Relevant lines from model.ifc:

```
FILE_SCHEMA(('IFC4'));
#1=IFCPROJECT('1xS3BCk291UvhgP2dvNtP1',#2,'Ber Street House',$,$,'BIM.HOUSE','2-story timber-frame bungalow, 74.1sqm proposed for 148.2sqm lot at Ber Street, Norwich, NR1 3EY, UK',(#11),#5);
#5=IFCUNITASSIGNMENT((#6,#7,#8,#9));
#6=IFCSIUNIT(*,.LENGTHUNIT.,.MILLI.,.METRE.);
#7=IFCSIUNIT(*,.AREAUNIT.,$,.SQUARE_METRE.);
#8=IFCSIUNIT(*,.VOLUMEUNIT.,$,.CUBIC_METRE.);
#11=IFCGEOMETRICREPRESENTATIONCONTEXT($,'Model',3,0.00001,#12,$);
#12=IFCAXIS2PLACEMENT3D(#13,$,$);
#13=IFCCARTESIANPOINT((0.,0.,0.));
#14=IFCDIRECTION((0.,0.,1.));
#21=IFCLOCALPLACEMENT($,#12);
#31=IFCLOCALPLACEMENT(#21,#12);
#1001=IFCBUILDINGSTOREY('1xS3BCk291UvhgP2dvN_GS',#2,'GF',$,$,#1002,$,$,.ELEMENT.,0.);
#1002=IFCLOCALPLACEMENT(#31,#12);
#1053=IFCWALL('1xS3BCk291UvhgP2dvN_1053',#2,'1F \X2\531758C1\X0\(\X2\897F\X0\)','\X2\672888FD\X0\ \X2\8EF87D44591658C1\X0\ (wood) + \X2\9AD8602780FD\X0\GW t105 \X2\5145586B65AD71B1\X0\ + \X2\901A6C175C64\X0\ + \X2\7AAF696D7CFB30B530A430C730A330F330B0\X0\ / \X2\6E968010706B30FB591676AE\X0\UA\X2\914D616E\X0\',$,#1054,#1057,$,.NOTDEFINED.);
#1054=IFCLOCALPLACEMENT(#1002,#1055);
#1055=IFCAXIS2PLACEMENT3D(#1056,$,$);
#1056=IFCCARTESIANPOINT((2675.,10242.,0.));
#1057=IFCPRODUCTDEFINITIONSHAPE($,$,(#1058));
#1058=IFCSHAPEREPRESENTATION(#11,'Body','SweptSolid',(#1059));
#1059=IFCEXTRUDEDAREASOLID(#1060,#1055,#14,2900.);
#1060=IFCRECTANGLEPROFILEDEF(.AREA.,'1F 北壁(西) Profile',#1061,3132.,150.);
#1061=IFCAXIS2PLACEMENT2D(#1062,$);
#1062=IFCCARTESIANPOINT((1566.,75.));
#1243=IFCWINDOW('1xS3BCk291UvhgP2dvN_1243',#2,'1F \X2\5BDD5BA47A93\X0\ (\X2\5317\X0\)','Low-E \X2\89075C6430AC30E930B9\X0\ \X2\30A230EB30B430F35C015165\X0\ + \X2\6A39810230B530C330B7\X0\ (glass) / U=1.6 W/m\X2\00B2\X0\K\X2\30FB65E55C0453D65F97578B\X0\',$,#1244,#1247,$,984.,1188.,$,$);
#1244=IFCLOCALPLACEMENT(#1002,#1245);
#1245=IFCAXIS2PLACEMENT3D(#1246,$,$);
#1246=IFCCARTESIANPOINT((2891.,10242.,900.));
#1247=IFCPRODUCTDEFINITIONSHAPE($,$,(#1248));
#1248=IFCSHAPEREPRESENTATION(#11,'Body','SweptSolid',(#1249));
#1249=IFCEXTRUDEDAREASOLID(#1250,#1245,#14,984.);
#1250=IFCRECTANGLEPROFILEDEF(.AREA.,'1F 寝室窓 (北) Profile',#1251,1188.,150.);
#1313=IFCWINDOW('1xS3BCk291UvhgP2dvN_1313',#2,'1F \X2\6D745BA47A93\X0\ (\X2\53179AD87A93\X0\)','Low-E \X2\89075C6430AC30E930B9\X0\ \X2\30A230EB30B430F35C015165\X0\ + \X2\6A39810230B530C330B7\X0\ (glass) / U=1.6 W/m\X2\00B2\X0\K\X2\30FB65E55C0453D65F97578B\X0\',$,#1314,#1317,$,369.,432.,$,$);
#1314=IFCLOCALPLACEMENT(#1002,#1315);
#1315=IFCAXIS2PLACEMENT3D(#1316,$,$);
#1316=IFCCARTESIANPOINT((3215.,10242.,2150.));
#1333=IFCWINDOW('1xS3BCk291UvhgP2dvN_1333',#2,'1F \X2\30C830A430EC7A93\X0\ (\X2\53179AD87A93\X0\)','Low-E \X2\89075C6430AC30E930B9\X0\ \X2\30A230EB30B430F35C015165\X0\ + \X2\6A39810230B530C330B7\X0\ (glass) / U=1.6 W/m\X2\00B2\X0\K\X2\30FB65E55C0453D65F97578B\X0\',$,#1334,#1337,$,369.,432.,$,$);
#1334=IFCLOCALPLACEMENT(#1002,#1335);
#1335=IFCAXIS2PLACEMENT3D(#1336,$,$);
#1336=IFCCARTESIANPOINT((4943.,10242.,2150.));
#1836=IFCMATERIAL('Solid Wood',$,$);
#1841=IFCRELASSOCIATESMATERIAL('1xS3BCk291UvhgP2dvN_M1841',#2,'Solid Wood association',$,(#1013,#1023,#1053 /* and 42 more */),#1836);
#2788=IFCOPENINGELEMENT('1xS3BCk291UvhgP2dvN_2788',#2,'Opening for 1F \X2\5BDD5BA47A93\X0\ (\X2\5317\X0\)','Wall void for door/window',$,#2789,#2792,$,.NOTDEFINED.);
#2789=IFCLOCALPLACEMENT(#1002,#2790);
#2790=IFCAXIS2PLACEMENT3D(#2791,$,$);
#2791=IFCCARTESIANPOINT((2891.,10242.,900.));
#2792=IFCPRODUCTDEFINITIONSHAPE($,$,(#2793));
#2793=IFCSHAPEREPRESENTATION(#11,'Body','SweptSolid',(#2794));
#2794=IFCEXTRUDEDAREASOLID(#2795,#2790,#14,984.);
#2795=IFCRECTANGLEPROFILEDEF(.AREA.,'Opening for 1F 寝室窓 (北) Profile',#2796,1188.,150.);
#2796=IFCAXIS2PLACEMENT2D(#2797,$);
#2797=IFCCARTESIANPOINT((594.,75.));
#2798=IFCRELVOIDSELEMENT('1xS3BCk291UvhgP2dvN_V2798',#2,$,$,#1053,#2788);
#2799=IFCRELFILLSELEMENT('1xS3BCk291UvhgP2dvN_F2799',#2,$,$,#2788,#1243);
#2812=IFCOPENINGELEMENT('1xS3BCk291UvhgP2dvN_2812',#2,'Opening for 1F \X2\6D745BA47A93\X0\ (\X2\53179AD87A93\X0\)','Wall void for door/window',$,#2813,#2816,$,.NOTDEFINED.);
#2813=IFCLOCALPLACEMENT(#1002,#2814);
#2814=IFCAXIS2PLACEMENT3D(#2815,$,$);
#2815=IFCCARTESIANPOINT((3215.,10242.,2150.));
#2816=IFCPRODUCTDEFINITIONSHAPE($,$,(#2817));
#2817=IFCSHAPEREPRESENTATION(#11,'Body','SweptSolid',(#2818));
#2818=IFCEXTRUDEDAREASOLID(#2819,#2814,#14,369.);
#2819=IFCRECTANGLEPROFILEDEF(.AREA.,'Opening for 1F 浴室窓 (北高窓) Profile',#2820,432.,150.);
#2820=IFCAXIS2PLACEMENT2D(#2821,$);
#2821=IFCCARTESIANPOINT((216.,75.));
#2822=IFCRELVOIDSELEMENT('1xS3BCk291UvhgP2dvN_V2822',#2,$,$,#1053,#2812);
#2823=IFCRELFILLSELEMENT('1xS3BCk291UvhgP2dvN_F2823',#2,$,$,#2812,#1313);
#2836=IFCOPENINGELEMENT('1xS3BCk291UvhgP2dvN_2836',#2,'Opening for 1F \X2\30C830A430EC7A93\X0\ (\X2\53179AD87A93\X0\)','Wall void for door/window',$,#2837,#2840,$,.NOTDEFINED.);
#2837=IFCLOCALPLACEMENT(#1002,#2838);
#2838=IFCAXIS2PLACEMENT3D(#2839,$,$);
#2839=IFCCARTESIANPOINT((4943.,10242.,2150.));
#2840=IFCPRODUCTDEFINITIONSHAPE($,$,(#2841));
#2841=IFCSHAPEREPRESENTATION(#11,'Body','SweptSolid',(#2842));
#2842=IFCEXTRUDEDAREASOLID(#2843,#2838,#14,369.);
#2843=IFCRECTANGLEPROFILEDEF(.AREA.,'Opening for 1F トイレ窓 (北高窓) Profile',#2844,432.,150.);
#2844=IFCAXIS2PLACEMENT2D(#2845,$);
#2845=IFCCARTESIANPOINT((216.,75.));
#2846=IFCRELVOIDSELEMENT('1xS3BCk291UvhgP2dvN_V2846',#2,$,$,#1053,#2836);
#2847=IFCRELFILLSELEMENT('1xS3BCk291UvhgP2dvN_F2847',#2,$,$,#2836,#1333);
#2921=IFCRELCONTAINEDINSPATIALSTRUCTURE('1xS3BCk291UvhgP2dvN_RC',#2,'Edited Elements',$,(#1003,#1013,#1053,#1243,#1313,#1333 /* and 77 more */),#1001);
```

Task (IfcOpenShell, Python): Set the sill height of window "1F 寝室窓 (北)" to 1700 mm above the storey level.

```python
import numpy as np
import ifcopenshell
import ifcopenshell.api.geometry
import ifcopenshell.geom
import ifcopenshell.util.element
import ifcopenshell.util.placement
import ifcopenshell.util.shape
import ifcopenshell.util.unit

model = ifcopenshell.open("model.ifc")
unit_scale = ifcopenshell.util.unit.calculate_unit_scale(model)

window = model.by_guid("1xS3BCk291UvhgP2dvN_1243")
opening = window.FillsVoids[0].RelatingOpeningElement
storey = ifcopenshell.util.element.get_container(window, ifc_class="IfcBuildingStorey")
level = ifcopenshell.util.placement.get_local_placement(storey.ObjectPlacement)[2, 3]

# The opening's origin need not be at the sill, so measure its lowest point.
shape = ifcopenshell.geom.create_shape(ifcopenshell.geom.settings(), opening)
bottom = ifcopenshell.util.shape.get_shape_bottom_elevation(shape, shape.geometry) / unit_scale
dz = level + 1.7 / unit_scale - bottom

shift = np.array([0.0, 0.0, dz])
# The window is not placed relative to its opening, so move both.
for product in (opening, window):
    matrix = ifcopenshell.util.placement.get_local_placement(product.ObjectPlacement)
    matrix[:3, 3] += shift
    ifcopenshell.api.geometry.edit_object_placement(model, product=product, matrix=matrix, is_si=False)

print(f"moved by {dz * unit_scale:+.3f} m")

model.write("model_rev.ifc")
```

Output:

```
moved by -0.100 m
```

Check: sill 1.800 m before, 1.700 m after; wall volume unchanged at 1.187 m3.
